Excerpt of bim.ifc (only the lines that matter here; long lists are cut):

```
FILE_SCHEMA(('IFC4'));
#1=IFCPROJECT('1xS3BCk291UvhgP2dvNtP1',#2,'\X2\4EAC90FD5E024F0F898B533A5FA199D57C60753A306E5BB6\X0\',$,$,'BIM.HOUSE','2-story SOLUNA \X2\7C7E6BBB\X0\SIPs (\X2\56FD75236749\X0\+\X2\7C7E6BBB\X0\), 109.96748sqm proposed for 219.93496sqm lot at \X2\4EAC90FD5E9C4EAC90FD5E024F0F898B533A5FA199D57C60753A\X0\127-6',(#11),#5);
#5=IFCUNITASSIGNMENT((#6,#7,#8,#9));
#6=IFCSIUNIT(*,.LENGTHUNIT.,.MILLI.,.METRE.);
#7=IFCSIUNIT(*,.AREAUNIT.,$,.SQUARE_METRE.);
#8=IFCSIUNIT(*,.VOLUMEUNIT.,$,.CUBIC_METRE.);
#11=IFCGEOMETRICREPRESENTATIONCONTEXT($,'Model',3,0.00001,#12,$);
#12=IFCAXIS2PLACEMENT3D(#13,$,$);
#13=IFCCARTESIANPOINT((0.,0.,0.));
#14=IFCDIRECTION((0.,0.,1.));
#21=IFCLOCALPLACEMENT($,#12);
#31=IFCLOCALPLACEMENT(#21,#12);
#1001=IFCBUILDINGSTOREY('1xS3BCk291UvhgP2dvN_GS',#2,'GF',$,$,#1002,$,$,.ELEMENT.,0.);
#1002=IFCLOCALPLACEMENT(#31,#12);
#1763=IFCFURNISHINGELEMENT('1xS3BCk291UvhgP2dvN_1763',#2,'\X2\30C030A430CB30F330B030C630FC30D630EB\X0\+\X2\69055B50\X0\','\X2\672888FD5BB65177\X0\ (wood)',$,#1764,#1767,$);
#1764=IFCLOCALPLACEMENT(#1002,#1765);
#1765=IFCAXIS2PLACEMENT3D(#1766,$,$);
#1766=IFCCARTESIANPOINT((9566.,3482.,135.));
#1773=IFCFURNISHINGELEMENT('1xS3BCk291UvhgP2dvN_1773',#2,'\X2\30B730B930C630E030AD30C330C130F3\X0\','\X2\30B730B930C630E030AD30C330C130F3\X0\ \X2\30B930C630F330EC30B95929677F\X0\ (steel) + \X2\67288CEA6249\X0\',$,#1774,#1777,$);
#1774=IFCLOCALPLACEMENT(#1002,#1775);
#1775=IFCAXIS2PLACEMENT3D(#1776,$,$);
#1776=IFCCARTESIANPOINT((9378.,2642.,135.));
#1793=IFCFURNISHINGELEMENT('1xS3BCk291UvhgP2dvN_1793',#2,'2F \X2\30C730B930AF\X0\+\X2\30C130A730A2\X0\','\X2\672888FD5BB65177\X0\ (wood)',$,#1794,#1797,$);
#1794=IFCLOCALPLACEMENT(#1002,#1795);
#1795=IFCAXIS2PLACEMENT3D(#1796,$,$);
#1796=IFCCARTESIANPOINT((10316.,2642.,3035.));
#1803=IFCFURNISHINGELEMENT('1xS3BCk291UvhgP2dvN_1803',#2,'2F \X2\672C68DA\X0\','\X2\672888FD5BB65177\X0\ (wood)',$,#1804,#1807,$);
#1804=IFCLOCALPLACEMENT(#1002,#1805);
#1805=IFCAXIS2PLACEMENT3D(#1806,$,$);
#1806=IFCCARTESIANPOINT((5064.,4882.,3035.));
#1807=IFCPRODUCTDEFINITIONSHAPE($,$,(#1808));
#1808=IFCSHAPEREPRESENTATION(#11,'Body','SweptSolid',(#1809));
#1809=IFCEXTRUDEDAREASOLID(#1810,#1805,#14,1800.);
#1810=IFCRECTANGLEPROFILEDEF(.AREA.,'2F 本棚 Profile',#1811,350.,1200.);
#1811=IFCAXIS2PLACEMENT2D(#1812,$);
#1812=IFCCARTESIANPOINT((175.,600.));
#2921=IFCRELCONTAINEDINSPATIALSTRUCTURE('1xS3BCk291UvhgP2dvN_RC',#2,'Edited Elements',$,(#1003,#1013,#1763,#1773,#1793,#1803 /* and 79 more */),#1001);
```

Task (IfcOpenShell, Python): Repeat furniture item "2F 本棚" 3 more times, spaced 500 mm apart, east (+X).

```python
import numpy as np
import ifcopenshell
import ifcopenshell.api.geometry
import ifcopenshell.api.root
import ifcopenshell.util.element
import ifcopenshell.util.placement
import ifcopenshell.util.unit

model = ifcopenshell.open("bim.ifc")
unit_scale = ifcopenshell.util.unit.calculate_unit_scale(model)


def reuse_history(source, copy):
    """copy_class also copies each property set's owner history, people and application; keep the originals."""
    for rel in copy.IsDefinedBy:
        if rel.is_a("IfcRelDefinesByProperties") and (history := rel.RelatingPropertyDefinition.OwnerHistory):
            rel.RelatingPropertyDefinition.OwnerHistory = source.OwnerHistory
            ifcopenshell.util.element.remove_deep2(model, history)


source = model.by_id(1803)
base = ifcopenshell.util.placement.get_local_placement(source.ObjectPlacement)
step = np.array([1.0, 0.0, 0.0]) * 0.5 / unit_scale

for i in range(1, 4):
    copy = ifcopenshell.api.root.copy_class(model, product=source)
    copy.Representation = ifcopenshell.util.element.copy_deep(
        model, source.Representation, exclude=["IfcGeometricRepresentationContext", "IfcRepresentationMap"]
    )
    reuse_history(source, copy)
    matrix = base.copy()
    matrix[:3, 3] += i * step
    print("added at", matrix[:3, 3].round(3) + 0.0)
    ifcopenshell.api.geometry.edit_object_placement(model, product=copy, matrix=matrix, is_si=False)

model.write("bim_rev.ifc")
```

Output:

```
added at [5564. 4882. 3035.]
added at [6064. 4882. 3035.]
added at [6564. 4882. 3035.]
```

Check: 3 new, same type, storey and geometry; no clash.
